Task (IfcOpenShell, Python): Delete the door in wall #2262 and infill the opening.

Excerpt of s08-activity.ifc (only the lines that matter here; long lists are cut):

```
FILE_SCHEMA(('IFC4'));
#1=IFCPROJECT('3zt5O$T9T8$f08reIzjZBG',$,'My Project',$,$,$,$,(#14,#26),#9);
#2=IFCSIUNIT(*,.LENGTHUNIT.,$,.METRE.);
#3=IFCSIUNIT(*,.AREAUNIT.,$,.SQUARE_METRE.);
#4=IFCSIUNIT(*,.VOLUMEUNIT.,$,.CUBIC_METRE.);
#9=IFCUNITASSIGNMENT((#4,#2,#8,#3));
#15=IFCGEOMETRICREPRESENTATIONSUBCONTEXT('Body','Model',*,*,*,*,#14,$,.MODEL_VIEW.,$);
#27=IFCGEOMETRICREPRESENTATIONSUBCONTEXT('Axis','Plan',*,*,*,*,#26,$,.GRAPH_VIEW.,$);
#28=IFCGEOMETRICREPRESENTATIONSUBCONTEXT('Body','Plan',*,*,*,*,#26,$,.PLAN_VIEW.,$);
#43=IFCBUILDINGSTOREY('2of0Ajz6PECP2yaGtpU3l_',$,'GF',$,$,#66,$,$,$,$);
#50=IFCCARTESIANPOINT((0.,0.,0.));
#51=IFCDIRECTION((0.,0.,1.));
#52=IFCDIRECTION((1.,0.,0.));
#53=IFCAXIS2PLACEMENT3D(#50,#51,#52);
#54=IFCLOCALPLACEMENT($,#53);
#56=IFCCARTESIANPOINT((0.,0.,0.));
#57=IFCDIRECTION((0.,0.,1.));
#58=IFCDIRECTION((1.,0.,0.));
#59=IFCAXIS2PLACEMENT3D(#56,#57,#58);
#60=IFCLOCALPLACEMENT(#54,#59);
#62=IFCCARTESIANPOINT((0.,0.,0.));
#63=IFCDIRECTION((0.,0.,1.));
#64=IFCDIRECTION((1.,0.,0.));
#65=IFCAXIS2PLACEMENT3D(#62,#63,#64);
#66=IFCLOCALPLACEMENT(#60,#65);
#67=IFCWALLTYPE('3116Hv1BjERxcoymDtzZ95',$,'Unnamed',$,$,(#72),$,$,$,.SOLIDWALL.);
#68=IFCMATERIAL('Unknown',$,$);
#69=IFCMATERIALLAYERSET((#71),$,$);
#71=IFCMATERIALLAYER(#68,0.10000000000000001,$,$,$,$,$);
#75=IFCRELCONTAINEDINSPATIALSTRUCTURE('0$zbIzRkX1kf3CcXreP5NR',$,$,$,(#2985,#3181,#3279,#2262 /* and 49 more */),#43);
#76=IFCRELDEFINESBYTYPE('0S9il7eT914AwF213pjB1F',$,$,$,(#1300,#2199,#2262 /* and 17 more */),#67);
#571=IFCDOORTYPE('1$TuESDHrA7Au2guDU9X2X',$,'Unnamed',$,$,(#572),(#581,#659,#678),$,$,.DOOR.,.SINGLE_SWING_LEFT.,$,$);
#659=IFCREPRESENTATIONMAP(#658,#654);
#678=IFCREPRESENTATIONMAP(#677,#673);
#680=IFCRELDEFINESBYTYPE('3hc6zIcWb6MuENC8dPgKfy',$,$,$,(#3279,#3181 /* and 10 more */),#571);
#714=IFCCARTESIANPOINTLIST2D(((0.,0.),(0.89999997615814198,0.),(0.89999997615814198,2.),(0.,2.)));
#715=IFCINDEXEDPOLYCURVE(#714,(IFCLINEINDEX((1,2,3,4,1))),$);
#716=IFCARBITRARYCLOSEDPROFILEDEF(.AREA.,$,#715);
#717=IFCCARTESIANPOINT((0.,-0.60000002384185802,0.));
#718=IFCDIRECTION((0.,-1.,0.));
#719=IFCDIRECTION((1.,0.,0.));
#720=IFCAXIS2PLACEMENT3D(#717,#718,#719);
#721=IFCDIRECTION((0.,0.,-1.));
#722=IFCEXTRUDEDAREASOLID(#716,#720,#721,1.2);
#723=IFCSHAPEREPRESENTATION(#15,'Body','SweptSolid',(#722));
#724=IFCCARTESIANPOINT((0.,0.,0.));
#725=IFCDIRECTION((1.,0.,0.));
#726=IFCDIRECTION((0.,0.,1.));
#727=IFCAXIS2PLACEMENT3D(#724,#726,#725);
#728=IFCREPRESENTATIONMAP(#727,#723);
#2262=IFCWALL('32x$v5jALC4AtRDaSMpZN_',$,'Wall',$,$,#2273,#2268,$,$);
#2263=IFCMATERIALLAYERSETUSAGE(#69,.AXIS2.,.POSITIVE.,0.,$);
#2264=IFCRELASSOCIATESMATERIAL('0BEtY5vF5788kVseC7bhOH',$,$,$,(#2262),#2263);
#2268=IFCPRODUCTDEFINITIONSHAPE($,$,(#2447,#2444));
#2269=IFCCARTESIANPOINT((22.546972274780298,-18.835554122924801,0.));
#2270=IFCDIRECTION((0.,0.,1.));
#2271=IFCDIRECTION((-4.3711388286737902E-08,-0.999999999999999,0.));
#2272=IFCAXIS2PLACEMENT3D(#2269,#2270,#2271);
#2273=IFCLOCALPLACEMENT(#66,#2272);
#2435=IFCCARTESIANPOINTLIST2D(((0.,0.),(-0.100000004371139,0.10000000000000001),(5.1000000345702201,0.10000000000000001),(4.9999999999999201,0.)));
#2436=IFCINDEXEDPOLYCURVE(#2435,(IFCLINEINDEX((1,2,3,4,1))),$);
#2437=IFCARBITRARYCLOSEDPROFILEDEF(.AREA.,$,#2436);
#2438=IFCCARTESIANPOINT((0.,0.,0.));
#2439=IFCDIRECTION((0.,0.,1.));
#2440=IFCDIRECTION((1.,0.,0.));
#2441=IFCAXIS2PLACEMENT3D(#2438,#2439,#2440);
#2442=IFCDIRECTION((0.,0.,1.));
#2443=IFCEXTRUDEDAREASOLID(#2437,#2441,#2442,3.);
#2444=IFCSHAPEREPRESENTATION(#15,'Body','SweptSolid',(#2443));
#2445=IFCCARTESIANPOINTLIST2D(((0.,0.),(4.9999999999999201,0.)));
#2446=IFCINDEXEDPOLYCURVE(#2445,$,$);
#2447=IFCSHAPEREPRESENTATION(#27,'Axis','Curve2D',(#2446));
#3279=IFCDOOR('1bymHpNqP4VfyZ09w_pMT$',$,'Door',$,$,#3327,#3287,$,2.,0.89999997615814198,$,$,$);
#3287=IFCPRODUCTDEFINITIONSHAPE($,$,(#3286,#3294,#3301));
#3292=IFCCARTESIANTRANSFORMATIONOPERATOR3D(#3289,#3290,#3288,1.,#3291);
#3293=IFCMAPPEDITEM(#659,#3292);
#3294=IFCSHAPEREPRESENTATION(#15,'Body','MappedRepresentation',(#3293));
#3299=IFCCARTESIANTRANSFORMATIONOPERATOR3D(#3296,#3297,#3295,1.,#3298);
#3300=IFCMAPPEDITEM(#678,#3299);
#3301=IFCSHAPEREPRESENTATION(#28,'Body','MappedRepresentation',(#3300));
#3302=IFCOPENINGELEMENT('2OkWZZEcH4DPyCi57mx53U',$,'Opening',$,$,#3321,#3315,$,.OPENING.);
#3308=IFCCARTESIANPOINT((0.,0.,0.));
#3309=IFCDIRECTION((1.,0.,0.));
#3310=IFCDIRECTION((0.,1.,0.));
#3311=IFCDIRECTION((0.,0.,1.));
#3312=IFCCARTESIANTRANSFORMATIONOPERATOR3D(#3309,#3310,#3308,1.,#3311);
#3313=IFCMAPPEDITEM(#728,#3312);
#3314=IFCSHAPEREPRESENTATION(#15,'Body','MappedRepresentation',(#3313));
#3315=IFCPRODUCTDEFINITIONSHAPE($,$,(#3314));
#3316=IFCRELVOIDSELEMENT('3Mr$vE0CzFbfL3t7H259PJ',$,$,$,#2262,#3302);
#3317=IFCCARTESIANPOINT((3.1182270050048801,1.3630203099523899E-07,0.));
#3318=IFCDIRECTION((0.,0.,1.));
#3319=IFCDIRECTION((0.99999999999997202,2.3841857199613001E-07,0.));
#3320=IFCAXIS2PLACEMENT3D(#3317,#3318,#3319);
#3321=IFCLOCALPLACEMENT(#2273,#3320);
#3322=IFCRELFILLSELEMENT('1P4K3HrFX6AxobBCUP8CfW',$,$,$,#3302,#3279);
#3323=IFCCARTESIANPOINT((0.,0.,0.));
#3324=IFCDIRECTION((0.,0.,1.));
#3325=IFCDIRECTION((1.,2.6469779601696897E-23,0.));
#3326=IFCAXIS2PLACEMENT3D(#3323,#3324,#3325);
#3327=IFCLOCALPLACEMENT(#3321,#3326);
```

```python
import ifcopenshell
import ifcopenshell.api.feature
import ifcopenshell.api.root
import ifcopenshell.geom
import ifcopenshell.util.shape

model = ifcopenshell.open("s08-activity.ifc")
settings = ifcopenshell.geom.settings()


def volume(element):
    """Net volume in cubic metres, openings subtracted."""
    shape = ifcopenshell.geom.create_shape(settings, element)
    return ifcopenshell.util.shape.get_volume(shape.geometry)


door = model.by_guid("1bymHpNqP4VfyZ09w_pMT$")
opening = door.FillsVoids[0].RelatingOpeningElement
wall = opening.VoidsElements[0].RelatingBuildingElement
before = volume(wall)

ifcopenshell.api.root.remove_product(model, product=door)
ifcopenshell.api.feature.remove_feature(model, feature=opening)

after = volume(wall)

print(f"wall volume {before:.3f} -> {after:.3f} m3")

model.write("s08-activity_updated.ifc")
```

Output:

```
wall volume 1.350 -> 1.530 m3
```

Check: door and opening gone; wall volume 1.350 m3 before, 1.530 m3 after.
